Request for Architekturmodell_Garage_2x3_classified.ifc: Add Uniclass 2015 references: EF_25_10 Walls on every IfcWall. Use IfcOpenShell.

First a look at what the model holds.

```python
import ifcopenshell

model = ifcopenshell.open("Architekturmodell_Garage_2x3_classified.ifc")
print(model.schema)
print("classifications:", [c.Name for c in model.by_type("IfcClassification")])
for ifc_class in ("IfcDoor", "IfcRoof", "IfcStair", "IfcWall", "IfcWindow"):
    print(ifc_class, len(model.by_type(ifc_class)))
```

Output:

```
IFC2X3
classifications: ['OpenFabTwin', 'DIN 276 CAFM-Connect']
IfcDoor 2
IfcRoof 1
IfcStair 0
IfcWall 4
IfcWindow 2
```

```python
import ifcopenshell
import ifcopenshell.api.classification

model = ifcopenshell.open("Architekturmodell_Garage_2x3_classified.ifc")

# IFC2X3 requires Source and Edition and has no link from the project to the system.
system = model.create_entity("IfcClassification", Source="NBS", Edition="2015", Name="Uniclass 2015")

codes = {
    "IfcWall": ("EF_25_10", "Walls"),
}
for ifc_class, (code, name) in codes.items():
    products = model.by_type(ifc_class)
    ifcopenshell.api.classification.add_reference(
        model, products=products, classification=system, identification=code, name=name
    )
    print(code, len(products))

model.write("Architekturmodell_Garage_2x3_classified-out.ifc")
```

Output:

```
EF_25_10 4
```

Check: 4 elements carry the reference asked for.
